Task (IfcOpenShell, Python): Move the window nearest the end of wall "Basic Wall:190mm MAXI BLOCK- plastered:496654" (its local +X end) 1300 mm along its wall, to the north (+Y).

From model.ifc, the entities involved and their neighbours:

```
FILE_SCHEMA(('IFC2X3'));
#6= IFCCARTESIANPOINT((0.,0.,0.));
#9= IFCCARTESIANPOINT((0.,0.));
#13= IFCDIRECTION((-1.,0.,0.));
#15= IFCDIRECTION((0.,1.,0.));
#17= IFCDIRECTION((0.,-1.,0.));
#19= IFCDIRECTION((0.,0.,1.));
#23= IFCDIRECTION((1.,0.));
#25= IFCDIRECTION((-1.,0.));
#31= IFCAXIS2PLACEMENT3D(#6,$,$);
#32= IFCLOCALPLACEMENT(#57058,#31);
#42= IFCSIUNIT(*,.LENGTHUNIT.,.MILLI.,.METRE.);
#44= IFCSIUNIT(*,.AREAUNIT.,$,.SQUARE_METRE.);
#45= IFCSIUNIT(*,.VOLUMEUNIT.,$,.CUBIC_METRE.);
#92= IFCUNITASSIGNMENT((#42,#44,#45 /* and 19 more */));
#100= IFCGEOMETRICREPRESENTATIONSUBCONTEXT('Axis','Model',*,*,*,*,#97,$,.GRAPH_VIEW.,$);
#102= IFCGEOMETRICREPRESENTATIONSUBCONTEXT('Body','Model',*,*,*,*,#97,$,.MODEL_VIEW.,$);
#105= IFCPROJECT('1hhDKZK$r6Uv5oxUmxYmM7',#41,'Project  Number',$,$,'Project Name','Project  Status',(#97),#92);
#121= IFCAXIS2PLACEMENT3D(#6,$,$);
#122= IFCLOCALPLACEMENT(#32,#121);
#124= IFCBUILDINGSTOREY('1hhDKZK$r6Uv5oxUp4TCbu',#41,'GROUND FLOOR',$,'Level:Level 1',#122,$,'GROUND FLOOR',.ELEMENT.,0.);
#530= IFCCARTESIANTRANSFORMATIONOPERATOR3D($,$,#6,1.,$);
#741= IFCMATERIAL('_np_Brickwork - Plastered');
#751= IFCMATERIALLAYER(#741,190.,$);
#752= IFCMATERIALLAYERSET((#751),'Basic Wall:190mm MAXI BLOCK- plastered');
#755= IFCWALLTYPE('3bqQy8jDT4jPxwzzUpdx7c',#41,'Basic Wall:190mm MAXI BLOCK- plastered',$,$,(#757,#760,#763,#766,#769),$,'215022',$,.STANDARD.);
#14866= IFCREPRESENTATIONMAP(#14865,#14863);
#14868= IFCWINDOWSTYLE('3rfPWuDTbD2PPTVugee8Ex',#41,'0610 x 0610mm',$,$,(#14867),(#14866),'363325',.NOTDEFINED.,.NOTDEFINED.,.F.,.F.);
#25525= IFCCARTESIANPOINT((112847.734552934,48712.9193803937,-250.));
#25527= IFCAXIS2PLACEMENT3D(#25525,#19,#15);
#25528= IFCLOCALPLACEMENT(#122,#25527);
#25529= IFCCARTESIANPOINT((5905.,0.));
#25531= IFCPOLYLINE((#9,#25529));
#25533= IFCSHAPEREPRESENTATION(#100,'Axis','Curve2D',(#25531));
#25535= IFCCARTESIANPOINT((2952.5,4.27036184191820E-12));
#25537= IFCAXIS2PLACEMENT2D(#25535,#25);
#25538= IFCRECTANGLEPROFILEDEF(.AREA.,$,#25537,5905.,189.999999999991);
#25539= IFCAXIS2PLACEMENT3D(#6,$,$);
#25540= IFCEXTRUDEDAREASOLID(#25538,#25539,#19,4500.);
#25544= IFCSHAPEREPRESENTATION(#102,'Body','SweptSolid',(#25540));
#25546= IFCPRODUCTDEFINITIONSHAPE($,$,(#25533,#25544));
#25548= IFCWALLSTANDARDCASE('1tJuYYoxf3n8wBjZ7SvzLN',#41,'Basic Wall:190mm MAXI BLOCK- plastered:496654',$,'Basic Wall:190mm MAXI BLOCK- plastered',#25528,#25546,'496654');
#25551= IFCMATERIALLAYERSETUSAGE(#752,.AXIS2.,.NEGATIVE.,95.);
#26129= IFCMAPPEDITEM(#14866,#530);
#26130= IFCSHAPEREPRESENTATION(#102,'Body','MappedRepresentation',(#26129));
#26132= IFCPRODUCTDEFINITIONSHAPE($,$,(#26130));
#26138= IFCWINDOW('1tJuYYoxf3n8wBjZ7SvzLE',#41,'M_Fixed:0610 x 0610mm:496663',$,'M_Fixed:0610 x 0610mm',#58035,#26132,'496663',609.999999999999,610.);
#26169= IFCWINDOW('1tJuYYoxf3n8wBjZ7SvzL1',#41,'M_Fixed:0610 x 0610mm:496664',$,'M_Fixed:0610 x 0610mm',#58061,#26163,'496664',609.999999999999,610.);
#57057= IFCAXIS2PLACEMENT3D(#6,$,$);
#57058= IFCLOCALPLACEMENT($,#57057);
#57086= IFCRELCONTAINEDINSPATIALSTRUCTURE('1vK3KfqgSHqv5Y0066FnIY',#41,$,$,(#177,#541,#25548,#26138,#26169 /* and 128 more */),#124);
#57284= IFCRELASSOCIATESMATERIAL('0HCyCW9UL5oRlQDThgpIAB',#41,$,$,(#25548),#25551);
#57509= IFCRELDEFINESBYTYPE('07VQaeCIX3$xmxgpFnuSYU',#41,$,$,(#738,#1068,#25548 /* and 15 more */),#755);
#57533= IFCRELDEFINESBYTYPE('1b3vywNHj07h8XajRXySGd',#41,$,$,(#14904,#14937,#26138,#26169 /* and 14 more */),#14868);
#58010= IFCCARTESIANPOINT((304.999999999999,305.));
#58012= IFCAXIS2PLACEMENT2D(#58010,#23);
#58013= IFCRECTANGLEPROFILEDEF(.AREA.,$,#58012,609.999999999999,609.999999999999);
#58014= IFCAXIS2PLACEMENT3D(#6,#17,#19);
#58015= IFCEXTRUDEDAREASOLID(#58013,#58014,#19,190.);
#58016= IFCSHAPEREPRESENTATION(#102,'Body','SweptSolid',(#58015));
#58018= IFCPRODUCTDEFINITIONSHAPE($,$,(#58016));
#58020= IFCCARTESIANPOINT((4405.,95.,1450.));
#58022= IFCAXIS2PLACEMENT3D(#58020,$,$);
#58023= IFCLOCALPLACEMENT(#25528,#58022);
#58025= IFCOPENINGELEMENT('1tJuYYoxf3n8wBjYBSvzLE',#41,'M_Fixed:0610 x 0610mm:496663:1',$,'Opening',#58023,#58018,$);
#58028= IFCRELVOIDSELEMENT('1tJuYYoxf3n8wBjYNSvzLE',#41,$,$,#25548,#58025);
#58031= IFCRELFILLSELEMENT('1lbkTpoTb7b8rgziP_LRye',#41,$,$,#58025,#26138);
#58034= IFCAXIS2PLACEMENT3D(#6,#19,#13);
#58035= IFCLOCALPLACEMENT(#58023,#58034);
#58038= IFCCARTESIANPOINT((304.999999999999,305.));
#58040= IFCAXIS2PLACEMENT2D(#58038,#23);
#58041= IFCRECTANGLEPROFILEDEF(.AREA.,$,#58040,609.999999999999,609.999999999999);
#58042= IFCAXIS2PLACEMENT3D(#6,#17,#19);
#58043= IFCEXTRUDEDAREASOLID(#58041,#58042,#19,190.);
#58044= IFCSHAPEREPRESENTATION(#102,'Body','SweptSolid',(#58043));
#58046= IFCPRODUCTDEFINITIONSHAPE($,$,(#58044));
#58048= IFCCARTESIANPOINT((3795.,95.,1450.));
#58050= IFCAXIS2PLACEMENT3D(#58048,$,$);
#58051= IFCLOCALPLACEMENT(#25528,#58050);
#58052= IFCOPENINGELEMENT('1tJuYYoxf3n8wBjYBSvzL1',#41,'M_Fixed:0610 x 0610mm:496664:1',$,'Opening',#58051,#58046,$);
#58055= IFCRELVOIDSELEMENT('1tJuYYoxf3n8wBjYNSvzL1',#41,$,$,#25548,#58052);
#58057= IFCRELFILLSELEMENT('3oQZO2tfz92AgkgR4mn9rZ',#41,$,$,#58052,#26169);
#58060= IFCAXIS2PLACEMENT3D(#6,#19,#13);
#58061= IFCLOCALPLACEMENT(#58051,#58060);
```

```python
import ifcopenshell
import ifcopenshell.api.geometry
import ifcopenshell.util.placement

model = ifcopenshell.open("model.ifc")

window = model.by_guid("1tJuYYoxf3n8wBjZ7SvzLE")
opening = window.FillsVoids[0].RelatingOpeningElement
wall = opening.VoidsElements[0].RelatingBuildingElement

wall_matrix = ifcopenshell.util.placement.get_local_placement(wall.ObjectPlacement)
shift = wall_matrix[:3, 0] * 1300.0
before = ifcopenshell.util.placement.get_local_placement(window.ObjectPlacement)[:3, 3].copy()

# The window is placed relative to its opening, so it follows when the opening moves.
matrix = ifcopenshell.util.placement.get_local_placement(opening.ObjectPlacement)
matrix[:3, 3] += shift
ifcopenshell.api.geometry.edit_object_placement(
    model, product=opening, matrix=matrix, is_si=False, should_transform_children=True
)

after = ifcopenshell.util.placement.get_local_placement(window.ObjectPlacement)[:3, 3]
print("window moved by", (after - before).round(3) + 0.0)

model.write("model-out.ifc")
```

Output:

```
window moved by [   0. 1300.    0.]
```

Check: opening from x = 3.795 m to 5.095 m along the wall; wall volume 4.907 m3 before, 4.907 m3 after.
